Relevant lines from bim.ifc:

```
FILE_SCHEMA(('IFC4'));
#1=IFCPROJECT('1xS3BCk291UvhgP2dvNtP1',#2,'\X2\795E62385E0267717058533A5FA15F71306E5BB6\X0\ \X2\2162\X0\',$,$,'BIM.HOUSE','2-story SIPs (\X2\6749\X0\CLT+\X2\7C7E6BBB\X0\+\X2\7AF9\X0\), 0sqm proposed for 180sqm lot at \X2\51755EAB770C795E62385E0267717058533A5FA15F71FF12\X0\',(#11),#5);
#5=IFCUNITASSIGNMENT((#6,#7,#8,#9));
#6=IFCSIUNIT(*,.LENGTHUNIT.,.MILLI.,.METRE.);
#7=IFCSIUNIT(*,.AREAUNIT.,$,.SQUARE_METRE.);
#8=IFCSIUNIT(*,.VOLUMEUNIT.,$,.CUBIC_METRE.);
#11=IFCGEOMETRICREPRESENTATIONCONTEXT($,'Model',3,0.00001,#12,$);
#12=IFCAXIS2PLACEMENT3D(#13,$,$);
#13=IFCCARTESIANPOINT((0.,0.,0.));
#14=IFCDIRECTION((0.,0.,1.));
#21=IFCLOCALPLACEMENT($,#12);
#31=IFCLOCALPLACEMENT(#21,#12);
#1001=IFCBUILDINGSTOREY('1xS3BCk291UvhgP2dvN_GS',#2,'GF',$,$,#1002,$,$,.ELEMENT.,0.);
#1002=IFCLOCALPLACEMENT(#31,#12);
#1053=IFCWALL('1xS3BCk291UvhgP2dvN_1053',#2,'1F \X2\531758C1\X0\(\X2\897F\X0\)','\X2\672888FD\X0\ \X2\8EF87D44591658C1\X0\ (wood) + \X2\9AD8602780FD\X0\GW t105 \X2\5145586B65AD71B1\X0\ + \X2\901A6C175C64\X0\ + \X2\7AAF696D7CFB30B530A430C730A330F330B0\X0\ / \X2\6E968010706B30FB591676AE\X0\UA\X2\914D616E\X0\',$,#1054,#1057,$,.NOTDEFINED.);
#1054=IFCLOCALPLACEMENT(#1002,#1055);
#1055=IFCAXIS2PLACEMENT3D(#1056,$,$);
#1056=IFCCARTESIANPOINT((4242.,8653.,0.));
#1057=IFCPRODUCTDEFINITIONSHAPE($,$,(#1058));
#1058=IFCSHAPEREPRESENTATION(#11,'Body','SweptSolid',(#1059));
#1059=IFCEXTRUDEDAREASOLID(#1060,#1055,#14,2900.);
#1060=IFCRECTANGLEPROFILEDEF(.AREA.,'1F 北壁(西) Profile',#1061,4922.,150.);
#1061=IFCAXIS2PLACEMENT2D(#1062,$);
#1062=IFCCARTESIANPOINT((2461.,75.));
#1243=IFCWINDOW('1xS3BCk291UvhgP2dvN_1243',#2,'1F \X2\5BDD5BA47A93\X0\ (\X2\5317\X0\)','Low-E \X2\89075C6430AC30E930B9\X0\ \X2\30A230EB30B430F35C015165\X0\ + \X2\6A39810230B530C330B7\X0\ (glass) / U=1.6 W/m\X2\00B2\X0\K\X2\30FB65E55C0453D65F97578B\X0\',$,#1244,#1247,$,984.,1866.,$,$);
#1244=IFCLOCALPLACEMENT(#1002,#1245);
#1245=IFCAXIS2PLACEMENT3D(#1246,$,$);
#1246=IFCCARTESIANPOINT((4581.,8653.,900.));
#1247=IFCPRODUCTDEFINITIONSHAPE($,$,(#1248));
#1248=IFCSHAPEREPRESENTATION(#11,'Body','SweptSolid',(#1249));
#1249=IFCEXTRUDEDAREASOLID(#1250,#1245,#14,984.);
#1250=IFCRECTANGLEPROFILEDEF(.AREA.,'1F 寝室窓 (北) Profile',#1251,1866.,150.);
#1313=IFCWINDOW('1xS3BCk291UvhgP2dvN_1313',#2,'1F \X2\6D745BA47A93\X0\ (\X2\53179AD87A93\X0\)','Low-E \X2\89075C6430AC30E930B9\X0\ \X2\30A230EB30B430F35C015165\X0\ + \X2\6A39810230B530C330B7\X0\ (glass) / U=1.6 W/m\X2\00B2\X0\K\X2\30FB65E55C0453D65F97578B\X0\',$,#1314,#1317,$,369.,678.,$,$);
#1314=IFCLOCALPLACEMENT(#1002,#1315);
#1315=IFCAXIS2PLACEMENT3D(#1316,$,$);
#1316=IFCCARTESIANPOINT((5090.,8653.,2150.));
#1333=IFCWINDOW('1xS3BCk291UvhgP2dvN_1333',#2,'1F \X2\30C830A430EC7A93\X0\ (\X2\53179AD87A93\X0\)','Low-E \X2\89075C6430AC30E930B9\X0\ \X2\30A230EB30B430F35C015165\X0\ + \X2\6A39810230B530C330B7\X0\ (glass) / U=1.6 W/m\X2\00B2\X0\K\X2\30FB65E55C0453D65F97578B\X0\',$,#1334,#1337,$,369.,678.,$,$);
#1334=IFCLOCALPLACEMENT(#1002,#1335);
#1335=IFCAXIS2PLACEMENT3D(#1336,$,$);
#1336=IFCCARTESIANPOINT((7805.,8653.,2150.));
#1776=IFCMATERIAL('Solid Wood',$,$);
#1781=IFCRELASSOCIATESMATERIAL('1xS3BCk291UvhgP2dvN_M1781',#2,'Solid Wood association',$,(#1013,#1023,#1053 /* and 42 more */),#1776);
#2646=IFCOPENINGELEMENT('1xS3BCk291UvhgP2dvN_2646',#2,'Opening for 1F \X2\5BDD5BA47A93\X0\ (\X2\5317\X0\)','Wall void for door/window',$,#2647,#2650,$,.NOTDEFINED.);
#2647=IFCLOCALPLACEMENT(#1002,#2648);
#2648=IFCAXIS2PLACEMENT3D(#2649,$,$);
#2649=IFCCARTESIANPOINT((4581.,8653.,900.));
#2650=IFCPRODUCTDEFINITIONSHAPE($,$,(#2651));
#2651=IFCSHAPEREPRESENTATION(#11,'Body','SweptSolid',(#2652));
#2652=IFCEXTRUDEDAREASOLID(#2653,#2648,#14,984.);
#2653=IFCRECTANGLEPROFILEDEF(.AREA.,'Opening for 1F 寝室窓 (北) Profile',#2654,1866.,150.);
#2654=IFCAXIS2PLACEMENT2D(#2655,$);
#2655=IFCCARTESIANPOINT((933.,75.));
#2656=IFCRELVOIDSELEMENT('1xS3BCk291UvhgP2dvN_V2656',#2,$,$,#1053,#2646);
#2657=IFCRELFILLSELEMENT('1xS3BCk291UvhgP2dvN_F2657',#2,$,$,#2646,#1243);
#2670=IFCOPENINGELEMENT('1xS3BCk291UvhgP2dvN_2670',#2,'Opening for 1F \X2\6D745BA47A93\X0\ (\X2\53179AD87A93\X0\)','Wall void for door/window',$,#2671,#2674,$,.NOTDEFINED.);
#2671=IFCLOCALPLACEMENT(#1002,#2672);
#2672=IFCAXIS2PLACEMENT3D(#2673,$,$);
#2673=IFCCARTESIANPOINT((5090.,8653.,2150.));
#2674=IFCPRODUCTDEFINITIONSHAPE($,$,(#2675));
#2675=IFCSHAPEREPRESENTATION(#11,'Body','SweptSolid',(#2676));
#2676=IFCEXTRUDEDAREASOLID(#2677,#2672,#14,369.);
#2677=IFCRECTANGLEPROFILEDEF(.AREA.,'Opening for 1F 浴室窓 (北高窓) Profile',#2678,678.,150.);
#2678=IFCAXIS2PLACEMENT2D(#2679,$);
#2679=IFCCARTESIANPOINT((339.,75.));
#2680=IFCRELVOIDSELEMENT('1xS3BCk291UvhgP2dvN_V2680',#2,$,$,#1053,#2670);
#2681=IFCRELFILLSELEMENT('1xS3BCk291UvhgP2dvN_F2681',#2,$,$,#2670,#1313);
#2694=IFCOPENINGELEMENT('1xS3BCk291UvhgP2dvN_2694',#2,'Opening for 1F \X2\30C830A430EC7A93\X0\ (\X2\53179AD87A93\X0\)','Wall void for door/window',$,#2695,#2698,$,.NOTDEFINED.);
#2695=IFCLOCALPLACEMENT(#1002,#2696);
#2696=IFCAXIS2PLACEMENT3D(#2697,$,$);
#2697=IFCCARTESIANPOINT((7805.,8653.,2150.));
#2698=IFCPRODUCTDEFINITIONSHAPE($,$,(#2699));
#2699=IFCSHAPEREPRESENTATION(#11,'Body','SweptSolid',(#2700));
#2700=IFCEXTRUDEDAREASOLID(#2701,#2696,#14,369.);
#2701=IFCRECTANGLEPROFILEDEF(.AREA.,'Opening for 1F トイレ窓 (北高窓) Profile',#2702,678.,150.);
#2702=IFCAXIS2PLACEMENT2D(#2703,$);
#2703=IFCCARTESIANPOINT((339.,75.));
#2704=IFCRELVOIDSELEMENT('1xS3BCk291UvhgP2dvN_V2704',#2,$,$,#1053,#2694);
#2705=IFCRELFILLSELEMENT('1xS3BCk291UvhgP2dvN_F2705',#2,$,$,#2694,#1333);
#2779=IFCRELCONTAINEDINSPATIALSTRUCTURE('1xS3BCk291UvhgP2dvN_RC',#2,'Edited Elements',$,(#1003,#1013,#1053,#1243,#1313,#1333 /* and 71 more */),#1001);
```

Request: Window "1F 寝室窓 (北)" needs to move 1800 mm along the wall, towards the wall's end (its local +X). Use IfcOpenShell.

```python
import ifcopenshell
import ifcopenshell.api.geometry
import ifcopenshell.util.placement
import ifcopenshell.util.unit

model = ifcopenshell.open("bim.ifc")
unit_scale = ifcopenshell.util.unit.calculate_unit_scale(model)

window = model.by_guid("1xS3BCk291UvhgP2dvN_1243")
opening = window.FillsVoids[0].RelatingOpeningElement
wall = opening.VoidsElements[0].RelatingBuildingElement

wall_matrix = ifcopenshell.util.placement.get_local_placement(wall.ObjectPlacement)
shift = wall_matrix[:3, 0] * 1.8 / unit_scale
before = ifcopenshell.util.placement.get_local_placement(window.ObjectPlacement)[:3, 3].copy()

# The window is not placed relative to its opening, so move both.
for product in (opening, window):
    matrix = ifcopenshell.util.placement.get_local_placement(product.ObjectPlacement)
    matrix[:3, 3] += shift
    ifcopenshell.api.geometry.edit_object_placement(model, product=product, matrix=matrix, is_si=False)

after = ifcopenshell.util.placement.get_local_placement(window.ObjectPlacement)[:3, 3]
print("window moved by", (after - before).round(3) + 0.0)

model.write("bim_rev.ifc")
```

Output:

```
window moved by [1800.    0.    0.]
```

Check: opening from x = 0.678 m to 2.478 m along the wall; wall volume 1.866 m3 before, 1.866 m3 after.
